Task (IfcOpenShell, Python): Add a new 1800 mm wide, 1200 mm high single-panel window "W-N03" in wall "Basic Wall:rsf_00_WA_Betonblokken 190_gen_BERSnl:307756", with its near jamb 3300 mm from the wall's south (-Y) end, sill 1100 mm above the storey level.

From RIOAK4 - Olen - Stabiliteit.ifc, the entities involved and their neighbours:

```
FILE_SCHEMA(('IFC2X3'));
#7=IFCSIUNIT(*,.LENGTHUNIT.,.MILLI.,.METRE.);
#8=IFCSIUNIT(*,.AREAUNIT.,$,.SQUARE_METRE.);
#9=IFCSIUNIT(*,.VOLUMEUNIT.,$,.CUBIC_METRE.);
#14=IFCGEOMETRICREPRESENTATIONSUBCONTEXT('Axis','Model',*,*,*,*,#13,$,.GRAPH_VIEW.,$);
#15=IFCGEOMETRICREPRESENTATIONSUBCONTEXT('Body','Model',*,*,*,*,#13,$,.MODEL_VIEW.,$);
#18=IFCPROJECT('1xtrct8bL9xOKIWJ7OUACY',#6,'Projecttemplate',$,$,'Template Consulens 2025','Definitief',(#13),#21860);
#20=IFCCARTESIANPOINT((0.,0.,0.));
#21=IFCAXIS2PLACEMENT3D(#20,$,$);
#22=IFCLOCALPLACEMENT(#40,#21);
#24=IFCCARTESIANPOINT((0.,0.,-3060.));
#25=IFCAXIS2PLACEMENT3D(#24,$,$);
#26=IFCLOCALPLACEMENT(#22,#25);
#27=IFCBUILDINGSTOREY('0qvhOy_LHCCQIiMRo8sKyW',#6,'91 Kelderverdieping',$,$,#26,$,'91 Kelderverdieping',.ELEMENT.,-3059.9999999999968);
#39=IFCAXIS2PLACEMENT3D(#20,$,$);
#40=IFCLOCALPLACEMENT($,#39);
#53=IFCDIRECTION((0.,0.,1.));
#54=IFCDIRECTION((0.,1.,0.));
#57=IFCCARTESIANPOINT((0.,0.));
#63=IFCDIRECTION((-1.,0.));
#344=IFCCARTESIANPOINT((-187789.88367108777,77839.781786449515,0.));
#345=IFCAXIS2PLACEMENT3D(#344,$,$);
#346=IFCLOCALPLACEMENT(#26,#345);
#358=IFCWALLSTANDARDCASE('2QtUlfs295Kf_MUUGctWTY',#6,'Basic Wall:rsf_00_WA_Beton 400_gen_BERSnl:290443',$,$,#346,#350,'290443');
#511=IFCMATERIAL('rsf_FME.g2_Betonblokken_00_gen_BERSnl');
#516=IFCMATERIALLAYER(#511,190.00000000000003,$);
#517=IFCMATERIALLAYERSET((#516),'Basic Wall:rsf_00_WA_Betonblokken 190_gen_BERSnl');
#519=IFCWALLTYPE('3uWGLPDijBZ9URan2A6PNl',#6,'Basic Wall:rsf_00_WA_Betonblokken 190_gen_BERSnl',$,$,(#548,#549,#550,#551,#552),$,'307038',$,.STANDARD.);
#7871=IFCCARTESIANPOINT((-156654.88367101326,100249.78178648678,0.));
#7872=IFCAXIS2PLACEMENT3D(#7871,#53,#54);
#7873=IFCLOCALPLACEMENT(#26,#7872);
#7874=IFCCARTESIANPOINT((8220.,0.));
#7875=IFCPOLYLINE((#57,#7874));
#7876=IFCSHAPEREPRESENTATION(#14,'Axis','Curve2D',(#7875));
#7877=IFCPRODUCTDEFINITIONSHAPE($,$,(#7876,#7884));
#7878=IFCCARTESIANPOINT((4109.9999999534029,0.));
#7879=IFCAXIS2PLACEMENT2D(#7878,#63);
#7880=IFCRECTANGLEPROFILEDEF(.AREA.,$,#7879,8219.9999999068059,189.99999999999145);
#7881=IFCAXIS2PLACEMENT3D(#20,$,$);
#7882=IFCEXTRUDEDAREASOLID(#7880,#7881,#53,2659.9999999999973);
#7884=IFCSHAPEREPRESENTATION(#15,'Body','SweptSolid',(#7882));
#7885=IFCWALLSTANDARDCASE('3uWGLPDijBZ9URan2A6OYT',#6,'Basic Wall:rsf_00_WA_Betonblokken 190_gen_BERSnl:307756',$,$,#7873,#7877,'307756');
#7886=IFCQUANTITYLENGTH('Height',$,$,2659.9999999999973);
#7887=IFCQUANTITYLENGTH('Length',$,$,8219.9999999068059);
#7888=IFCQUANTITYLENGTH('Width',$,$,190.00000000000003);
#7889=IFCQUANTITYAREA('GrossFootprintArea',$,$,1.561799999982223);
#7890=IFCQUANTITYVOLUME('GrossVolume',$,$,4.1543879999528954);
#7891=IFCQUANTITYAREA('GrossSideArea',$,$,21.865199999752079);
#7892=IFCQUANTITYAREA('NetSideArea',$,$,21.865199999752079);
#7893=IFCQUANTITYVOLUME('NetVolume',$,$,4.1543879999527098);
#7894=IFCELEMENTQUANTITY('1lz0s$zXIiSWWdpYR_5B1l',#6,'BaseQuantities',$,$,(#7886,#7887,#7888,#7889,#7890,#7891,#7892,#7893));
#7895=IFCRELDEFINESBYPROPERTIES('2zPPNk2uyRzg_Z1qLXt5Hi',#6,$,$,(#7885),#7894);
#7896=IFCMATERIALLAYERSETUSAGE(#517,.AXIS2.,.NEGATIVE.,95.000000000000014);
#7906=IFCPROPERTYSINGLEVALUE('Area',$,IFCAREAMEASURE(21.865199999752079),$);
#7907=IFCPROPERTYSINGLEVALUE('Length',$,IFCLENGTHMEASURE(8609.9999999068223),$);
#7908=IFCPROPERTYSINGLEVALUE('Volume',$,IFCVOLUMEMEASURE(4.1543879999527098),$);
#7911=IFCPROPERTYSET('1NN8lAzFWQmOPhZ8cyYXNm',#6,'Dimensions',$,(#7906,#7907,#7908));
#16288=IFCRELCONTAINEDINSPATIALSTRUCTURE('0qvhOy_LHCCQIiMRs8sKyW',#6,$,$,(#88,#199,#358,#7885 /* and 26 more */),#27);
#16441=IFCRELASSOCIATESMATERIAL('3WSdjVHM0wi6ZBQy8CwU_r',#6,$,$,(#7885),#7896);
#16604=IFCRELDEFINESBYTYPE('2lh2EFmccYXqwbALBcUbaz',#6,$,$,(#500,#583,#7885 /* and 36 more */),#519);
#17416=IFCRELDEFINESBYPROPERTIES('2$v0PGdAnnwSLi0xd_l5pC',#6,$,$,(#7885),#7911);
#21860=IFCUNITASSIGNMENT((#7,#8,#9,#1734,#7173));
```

```python
import numpy as np
import ifcopenshell
import ifcopenshell.api.feature
import ifcopenshell.api.geometry
import ifcopenshell.api.pset
import ifcopenshell.api.root
import ifcopenshell.api.spatial
import ifcopenshell.api.type
import ifcopenshell.geom
import ifcopenshell.util.element
import ifcopenshell.util.placement
import ifcopenshell.util.representation
import ifcopenshell.util.shape
import ifcopenshell.util.unit

model = ifcopenshell.open("RIOAK4 - Olen - Stabiliteit.ifc")
unit_scale = ifcopenshell.util.unit.calculate_unit_scale(model)
area_scale = ifcopenshell.util.unit.calculate_unit_scale(model, "AREAUNIT")
volume_scale = ifcopenshell.util.unit.calculate_unit_scale(model, "VOLUMEUNIT")
settings = ifcopenshell.geom.settings()


def volume(element):
    """Net volume in cubic metres, openings subtracted."""
    shape = ifcopenshell.geom.create_shape(settings, element)
    return ifcopenshell.util.shape.get_volume(shape.geometry)


wall = model.by_id(7885)
storey = ifcopenshell.util.element.get_container(wall, ifc_class="IfcBuildingStorey")
context = ifcopenshell.util.representation.get_context(model, "Model", "Body", "MODEL_VIEW")
before = volume(wall)

width, height, from_end, sill = 1.8, 1.2, 3.3, 1.1  # metres

# The wall runs along its own X axis, and the end named is its -X end.
wall_shape = ifcopenshell.geom.create_shape(settings, wall)
x, y, z = ifcopenshell.util.shape.get_vertices(wall_shape.geometry).T
start = x.min() + from_end
face, thickness = float(y.min()), float(y.max() - y.min())
wall_matrix = ifcopenshell.util.placement.get_local_placement(wall.ObjectPlacement)
level = ifcopenshell.util.placement.get_local_placement(storey.ObjectPlacement)[2, 3]


def in_wall(x, y):
    """Placement at x, y metres in the wall's axes, at sill height."""
    matrix = wall_matrix.copy()
    matrix[:, 3] = wall_matrix @ np.array([x / unit_scale, y / unit_scale, 0.0, 1.0])
    matrix[2, 3] = level + sill / unit_scale
    return matrix


# Opening: a box that overshoots both wall faces by 50 mm.
opening = ifcopenshell.api.root.create_entity(model, ifc_class="IfcOpeningElement")
box = ifcopenshell.api.geometry.add_wall_representation(
    model, context=context, length=width, height=height, thickness=thickness + 0.1
)
ifcopenshell.api.geometry.assign_representation(model, product=opening, representation=box)
ifcopenshell.api.geometry.edit_object_placement(model, product=opening, matrix=in_wall(start, face - 0.05), is_si=False)
ifcopenshell.api.feature.add_feature(model, feature=opening, element=wall)

window = ifcopenshell.api.root.create_entity(model, ifc_class="IfcWindow", name="W-N03")
window.OverallWidth, window.OverallHeight = width / unit_scale, height / unit_scale
body = ifcopenshell.api.geometry.add_window_representation(
    model,
    context=context,
    overall_width=window.OverallWidth,
    overall_height=window.OverallHeight,
    partition_type="SINGLE_PANEL",
)
ifcopenshell.api.geometry.assign_representation(model, product=window, representation=body)
ifcopenshell.api.spatial.assign_container(model, products=[window], relating_structure=storey)
fills = ifcopenshell.api.feature.add_filling(model, opening=opening, element=window)
fills.OwnerHistory = window.OwnerHistory  # required in IFC2X3

# IFC2X3 keeps the operation on the window style.
style = ifcopenshell.api.root.create_entity(model, ifc_class="IfcWindowStyle", name="W-N03")
style.OperationType, style.ConstructionType = "SINGLE_PANEL", "NOTDEFINED"
style.ParameterTakesPrecedence = style.Sizeable = False
ifcopenshell.api.type.assign_type(model, related_objects=[window], relating_type=style)

# Centre the window in the wall's thickness.
ifcopenshell.api.geometry.edit_object_placement(model, product=window, matrix=in_wall(start, face), is_si=False)
window_shape = ifcopenshell.geom.create_shape(settings, window)
depth = ifcopenshell.util.shape.get_vertices(window_shape.geometry)[:, 1]
offset = face + thickness / 2 - (depth.min() + depth.max()) / 2
ifcopenshell.api.geometry.edit_object_placement(model, product=window, matrix=in_wall(start, offset), is_si=False)

after = volume(wall)

# Update the wall's stored quantities.
qto = model.by_id(ifcopenshell.util.element.get_pset(wall, "BaseQuantities", should_inherit=False)["id"])
ifcopenshell.api.pset.edit_qto(model, qto=qto, properties={
    "NetSideArea": after / thickness / area_scale,
    "NetVolume": after / volume_scale,
})
pset = model.by_id(ifcopenshell.util.element.get_pset(wall, "Dimensions", should_inherit=False)["id"])
ifcopenshell.api.pset.edit_pset(model, pset=pset, properties={
    "Area": model.create_entity("IfcAreaMeasure", after / thickness / area_scale),
    "Volume": model.create_entity("IfcVolumeMeasure", after / volume_scale),
})

print(f"wall volume {before:.3f} -> {after:.3f} m3")

model.write("RIOAK4 - Olen - Stabiliteit_v2.ifc")
```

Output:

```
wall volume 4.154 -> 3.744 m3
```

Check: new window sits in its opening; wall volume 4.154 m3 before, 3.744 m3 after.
